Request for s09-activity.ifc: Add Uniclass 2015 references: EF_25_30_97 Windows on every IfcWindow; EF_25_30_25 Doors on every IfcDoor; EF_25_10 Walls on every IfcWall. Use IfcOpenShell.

First a look at what the model holds.

```python
import ifcopenshell

model = ifcopenshell.open("s09-activity.ifc")
print(model.schema)
print("classifications:", [c.Name for c in model.by_type("IfcClassification")])
for ifc_class in ("IfcDoor", "IfcRoof", "IfcStair", "IfcWall", "IfcWindow"):
    print(ifc_class, len(model.by_type(ifc_class)))
```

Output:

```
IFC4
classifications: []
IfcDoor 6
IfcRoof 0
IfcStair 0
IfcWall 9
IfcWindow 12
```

```python
import ifcopenshell
import ifcopenshell.api.classification

model = ifcopenshell.open("s09-activity.ifc")

system = ifcopenshell.api.classification.add_classification(model, classification="Uniclass 2015")

codes = {
    "IfcWindow": ("EF_25_30_97", "Windows"),
    "IfcDoor": ("EF_25_30_25", "Doors"),
    "IfcWall": ("EF_25_10", "Walls"),
}
for ifc_class, (code, name) in codes.items():
    products = model.by_type(ifc_class)
    ifcopenshell.api.classification.add_reference(
        model, products=products, classification=system, identification=code, name=name
    )
    print(code, len(products))

model.write("s09-activity_edited.ifc")
```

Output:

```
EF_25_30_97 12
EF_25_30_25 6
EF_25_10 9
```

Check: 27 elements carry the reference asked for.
